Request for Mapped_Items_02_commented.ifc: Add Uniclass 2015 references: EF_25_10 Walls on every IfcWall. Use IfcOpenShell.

First a look at what the model holds.

```python
import ifcopenshell

model = ifcopenshell.open("Mapped_Items_02_commented.ifc")
print(model.schema)
print("classifications:", [c.Name for c in model.by_type("IfcClassification")])
for ifc_class in ("IfcDoor", "IfcRoof", "IfcStair", "IfcWall", "IfcWindow"):
    print(ifc_class, len(model.by_type(ifc_class)))
```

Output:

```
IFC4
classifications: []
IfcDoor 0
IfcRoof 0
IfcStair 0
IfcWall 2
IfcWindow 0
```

```python
import ifcopenshell
import ifcopenshell.api.classification

model = ifcopenshell.open("Mapped_Items_02_commented.ifc")

system = ifcopenshell.api.classification.add_classification(model, classification="Uniclass 2015")

codes = {
    "IfcWall": ("EF_25_10", "Walls"),
}
for ifc_class, (code, name) in codes.items():
    products = model.by_type(ifc_class)
    ifcopenshell.api.classification.add_reference(
        model, products=products, classification=system, identification=code, name=name
    )
    print(code, len(products))

model.write("Mapped_Items_02_commented_v2.ifc")
```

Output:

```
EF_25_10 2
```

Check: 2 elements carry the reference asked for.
